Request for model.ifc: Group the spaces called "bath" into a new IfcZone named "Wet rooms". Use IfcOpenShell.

First a look at what the model holds.

```python
import ifcopenshell

model = ifcopenshell.open("model.ifc")
print(model.schema)
seen = {}
for space in model.by_type("IfcSpace"):
    seen[space.LongName] = seen.get(space.LongName, 0) + 1
for name, count in sorted(seen.items(), key=str):
    print(count, "x", name)
print("zones:", [z.Name for z in model.by_type("IfcZone")][:20])
```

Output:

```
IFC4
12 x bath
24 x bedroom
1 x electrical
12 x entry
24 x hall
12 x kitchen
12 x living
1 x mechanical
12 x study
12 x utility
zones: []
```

```python
import ifcopenshell
import ifcopenshell.api.group
import ifcopenshell.api.root

model = ifcopenshell.open("model.ifc")

names = {"bath"}
spaces = [s for s in model.by_type("IfcSpace") if s.LongName in names]

zone = ifcopenshell.api.root.create_entity(model, ifc_class="IfcZone", name="Wet rooms")
ifcopenshell.api.group.assign_group(model, products=spaces, group=zone)
print(len(spaces), "spaces in", zone.Name)

model.write("model-out.ifc")
```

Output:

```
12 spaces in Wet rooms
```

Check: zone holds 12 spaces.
